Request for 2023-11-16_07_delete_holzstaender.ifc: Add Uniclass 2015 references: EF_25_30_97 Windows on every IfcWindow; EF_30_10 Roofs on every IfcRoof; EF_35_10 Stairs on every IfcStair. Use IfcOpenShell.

First a look at what the model holds.

```python
import ifcopenshell

model = ifcopenshell.open("2023-11-16_07_delete_holzstaender.ifc")
print(model.schema)
print("classifications:", [c.Name for c in model.by_type("IfcClassification")])
for ifc_class in ("IfcDoor", "IfcRoof", "IfcStair", "IfcWall", "IfcWindow"):
    print(ifc_class, len(model.by_type(ifc_class)))
```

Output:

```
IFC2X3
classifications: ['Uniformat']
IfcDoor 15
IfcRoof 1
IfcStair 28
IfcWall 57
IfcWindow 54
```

```python
import ifcopenshell
import ifcopenshell.api.classification

model = ifcopenshell.open("2023-11-16_07_delete_holzstaender.ifc")

# IFC2X3 requires Source and Edition and has no link from the project to the system.
system = model.create_entity("IfcClassification", Source="NBS", Edition="2015", Name="Uniclass 2015")

codes = {
    "IfcWindow": ("EF_25_30_97", "Windows"),
    "IfcRoof": ("EF_30_10", "Roofs"),
    "IfcStair": ("EF_35_10", "Stairs"),
}
for ifc_class, (code, name) in codes.items():
    products = model.by_type(ifc_class)
    ifcopenshell.api.classification.add_reference(
        model, products=products, classification=system, identification=code, name=name
    )
    print(code, len(products))

model.write("2023-11-16_07_delete_holzstaender-out.ifc")
```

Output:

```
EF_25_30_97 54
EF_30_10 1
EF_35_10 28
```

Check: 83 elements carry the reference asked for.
